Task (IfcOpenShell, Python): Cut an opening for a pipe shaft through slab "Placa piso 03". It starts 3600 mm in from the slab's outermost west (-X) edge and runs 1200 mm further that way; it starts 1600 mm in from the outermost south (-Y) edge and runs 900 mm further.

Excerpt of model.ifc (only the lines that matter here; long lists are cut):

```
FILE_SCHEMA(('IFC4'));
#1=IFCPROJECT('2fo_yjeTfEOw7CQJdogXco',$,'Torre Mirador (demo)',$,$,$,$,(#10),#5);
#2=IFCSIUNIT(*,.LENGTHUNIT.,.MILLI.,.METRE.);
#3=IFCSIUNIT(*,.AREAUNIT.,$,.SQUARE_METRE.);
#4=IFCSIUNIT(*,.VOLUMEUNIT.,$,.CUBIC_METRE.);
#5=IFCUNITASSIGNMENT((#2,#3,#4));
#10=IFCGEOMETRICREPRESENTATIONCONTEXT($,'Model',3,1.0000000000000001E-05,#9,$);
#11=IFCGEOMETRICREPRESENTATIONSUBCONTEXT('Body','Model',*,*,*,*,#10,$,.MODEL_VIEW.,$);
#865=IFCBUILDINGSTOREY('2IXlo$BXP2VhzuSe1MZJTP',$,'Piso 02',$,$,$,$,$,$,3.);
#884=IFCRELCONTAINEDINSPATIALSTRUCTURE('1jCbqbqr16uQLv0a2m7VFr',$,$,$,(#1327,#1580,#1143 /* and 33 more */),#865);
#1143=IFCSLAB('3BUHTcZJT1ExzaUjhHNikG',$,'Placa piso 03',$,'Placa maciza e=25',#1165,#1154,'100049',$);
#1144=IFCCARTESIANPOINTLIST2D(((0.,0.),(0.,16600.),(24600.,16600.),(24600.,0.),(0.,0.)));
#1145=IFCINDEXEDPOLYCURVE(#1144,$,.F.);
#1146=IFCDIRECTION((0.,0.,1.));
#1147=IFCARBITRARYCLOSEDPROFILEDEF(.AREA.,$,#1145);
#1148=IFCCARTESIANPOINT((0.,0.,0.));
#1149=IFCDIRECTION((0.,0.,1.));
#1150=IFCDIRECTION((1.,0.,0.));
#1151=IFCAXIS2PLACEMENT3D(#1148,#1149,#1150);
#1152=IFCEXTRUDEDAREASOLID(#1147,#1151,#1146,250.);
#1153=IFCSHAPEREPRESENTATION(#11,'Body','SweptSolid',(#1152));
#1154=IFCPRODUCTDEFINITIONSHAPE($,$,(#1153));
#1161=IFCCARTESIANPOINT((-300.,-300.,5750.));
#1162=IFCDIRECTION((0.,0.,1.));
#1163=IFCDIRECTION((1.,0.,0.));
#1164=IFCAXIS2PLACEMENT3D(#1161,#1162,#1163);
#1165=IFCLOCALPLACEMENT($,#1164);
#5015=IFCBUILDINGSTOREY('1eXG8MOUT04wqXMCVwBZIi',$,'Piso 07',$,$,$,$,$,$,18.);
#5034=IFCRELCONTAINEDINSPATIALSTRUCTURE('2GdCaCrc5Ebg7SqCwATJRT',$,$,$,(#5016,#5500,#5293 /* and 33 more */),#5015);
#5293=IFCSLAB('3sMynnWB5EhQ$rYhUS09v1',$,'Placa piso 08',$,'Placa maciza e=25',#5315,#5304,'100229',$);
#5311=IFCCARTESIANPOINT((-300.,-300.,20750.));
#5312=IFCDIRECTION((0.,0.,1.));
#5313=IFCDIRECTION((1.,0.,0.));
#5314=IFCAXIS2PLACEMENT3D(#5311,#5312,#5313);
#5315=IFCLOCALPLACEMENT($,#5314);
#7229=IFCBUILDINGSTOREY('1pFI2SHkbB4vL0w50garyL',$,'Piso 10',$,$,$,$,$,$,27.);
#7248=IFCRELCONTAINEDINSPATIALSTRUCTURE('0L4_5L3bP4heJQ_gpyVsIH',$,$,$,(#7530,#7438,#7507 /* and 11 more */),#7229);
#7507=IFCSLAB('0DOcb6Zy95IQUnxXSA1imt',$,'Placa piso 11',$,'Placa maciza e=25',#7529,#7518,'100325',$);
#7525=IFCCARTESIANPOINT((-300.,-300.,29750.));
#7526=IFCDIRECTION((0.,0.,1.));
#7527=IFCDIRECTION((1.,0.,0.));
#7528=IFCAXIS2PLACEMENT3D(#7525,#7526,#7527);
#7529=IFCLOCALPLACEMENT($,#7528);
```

```python
import numpy as np
import ifcopenshell
import ifcopenshell.api.feature
import ifcopenshell.api.geometry
import ifcopenshell.api.root
import ifcopenshell.geom
import ifcopenshell.util.placement
import ifcopenshell.util.representation
import ifcopenshell.util.shape
import ifcopenshell.util.unit

model = ifcopenshell.open("model.ifc")
unit_scale = ifcopenshell.util.unit.calculate_unit_scale(model)
settings = ifcopenshell.geom.settings()


def volume(element):
    """Net volume in cubic metres, openings subtracted."""
    shape = ifcopenshell.geom.create_shape(settings, element)
    return ifcopenshell.util.shape.get_volume(shape.geometry)


slab = model.by_guid("3BUHTcZJT1ExzaUjhHNikG")
before = volume(slab)

# Extent in the slab's own axes, in metres. The edges named are its -X and -Y sides.
slab_shape = ifcopenshell.geom.create_shape(settings, slab)
vertices = ifcopenshell.util.shape.get_vertices(slab_shape.geometry)
x_min, y_min, bottom = vertices.min(axis=0)
top = vertices[:, 2].max()

opening = ifcopenshell.api.root.create_entity(model, ifc_class="IfcOpeningElement", name="Pipe shaft opening", predefined_type="OPENING")
context = ifcopenshell.util.representation.get_context(model, "Model", "Body", "MODEL_VIEW")
width, depth = 1.2, 0.9
outline = [(0.0, 0.0), (width, 0.0), (width, depth), (0.0, depth), (0.0, 0.0)]
# Overshoot both faces by 50 mm so the cut is clean.
shape = ifcopenshell.api.geometry.add_slab_representation(
    model, context=context, depth=top - bottom + 0.1, polyline=outline
)
ifcopenshell.api.geometry.assign_representation(model, product=opening, representation=shape)

matrix = ifcopenshell.util.placement.get_local_placement(slab.ObjectPlacement)
matrix[:, 3] = matrix @ np.append(np.array([x_min + 3.6, y_min + 1.6, bottom - 0.05]) / unit_scale, 1.0)
ifcopenshell.api.geometry.edit_object_placement(model, product=opening, matrix=matrix, is_si=False)
ifcopenshell.api.feature.add_feature(model, feature=opening, element=slab)

after = volume(slab)

print(f"slab volume {before:.3f} -> {after:.3f} m3")

model.write("model_updated.ifc")
```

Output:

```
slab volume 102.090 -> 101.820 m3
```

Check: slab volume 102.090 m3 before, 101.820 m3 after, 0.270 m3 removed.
